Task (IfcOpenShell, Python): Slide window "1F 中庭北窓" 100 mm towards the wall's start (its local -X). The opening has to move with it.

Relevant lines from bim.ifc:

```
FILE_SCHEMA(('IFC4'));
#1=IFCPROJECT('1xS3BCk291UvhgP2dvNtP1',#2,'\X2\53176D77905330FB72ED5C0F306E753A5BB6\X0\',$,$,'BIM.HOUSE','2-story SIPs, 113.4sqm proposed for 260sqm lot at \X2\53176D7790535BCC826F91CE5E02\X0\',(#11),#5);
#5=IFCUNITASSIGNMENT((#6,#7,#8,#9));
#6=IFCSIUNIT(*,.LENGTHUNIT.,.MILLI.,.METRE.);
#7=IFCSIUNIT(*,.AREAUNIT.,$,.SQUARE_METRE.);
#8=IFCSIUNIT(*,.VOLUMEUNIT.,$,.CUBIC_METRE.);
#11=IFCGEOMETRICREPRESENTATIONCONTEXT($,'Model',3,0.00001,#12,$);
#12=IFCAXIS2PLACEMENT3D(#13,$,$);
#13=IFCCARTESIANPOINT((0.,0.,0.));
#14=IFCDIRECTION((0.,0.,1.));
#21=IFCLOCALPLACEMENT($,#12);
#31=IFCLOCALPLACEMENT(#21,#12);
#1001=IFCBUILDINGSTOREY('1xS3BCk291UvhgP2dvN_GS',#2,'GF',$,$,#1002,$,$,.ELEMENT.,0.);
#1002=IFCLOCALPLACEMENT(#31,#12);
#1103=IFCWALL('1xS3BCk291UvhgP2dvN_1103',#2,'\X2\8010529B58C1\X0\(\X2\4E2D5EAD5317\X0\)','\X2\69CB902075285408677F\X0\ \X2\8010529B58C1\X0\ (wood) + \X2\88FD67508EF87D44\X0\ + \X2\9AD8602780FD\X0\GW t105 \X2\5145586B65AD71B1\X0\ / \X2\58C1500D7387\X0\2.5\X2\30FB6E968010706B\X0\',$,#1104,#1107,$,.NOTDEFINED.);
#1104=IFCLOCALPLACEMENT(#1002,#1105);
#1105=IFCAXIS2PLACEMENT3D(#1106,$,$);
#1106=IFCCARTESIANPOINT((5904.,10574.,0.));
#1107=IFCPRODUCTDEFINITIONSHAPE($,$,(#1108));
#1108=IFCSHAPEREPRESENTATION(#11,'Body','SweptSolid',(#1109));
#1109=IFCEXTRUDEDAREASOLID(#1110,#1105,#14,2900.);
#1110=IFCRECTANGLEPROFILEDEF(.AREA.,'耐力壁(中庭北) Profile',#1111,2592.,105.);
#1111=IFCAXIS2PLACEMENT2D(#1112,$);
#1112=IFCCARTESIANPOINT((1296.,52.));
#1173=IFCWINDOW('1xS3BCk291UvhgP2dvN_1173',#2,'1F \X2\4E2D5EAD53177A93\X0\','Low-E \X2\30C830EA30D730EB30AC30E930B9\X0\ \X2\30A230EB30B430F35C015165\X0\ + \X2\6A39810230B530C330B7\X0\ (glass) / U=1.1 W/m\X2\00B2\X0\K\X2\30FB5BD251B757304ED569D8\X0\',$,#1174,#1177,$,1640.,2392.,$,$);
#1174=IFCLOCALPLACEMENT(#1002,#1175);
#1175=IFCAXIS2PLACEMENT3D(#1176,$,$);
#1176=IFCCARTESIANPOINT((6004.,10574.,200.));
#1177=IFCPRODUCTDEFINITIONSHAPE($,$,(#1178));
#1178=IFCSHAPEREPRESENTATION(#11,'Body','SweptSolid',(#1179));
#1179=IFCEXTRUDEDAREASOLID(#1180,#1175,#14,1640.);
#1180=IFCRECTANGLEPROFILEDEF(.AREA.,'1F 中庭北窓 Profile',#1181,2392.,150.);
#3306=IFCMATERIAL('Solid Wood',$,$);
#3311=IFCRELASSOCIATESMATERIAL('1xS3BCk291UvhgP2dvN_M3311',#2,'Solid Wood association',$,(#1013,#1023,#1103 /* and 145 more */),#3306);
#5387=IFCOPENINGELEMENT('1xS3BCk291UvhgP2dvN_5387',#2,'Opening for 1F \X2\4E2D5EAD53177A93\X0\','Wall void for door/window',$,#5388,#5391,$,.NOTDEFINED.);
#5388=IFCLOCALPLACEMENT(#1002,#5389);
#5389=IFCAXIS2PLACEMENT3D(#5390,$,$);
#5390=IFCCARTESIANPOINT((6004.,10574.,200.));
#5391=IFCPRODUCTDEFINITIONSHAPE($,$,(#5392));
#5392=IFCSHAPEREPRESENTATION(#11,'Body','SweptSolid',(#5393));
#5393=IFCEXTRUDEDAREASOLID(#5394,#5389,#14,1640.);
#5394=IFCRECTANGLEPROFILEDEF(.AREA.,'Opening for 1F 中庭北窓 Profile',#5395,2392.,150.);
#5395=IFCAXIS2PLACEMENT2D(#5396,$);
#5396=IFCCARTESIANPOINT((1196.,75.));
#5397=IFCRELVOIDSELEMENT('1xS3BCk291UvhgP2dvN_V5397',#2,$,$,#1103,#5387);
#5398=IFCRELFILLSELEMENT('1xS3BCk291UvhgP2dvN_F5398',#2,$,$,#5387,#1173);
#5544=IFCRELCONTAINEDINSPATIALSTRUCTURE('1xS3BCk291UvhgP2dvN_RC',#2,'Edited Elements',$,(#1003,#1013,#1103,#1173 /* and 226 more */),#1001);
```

```python
import ifcopenshell
import ifcopenshell.api.geometry
import ifcopenshell.util.placement

model = ifcopenshell.open("bim.ifc")

window = model.by_guid("1xS3BCk291UvhgP2dvN_1173")
opening = window.FillsVoids[0].RelatingOpeningElement
wall = opening.VoidsElements[0].RelatingBuildingElement

wall_matrix = ifcopenshell.util.placement.get_local_placement(wall.ObjectPlacement)
shift = wall_matrix[:3, 0] * -100.0
before = ifcopenshell.util.placement.get_local_placement(window.ObjectPlacement)[:3, 3].copy()

# The window is not placed relative to its opening, so move both.
for product in (opening, window):
    matrix = ifcopenshell.util.placement.get_local_placement(product.ObjectPlacement)
    matrix[:3, 3] += shift
    ifcopenshell.api.geometry.edit_object_placement(model, product=product, matrix=matrix, is_si=False)

after = ifcopenshell.util.placement.get_local_placement(window.ObjectPlacement)[:3, 3]
print("window moved by", (after - before).round(3) + 0.0)

model.write("bim_v2.ifc")
```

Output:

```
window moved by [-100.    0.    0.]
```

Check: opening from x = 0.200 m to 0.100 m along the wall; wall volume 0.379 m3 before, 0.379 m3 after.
